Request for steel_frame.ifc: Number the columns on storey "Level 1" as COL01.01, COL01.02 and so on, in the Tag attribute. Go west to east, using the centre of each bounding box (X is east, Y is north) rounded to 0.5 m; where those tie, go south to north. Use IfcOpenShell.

First a look at what the model holds.

```python
import ifcopenshell
import ifcopenshell.util.element
import ifcopenshell.util.placement

model = ifcopenshell.open("steel_frame.ifc")
print(model.schema)
storey = next(s for s in model.by_type("IfcBuildingStorey") if s.Name == "Level 1")
columns = [e for e in ifcopenshell.util.element.get_decomposition(storey) if e.is_a("IfcColumn")]
for e in sorted(columns, key=lambda e: e.id()):
    origin = ifcopenshell.util.placement.get_local_placement(e.ObjectPlacement)[:3, 3]
    print(e.id(), e.Tag, e.Name, origin.round(2) + 0.0, sep=" | ")
```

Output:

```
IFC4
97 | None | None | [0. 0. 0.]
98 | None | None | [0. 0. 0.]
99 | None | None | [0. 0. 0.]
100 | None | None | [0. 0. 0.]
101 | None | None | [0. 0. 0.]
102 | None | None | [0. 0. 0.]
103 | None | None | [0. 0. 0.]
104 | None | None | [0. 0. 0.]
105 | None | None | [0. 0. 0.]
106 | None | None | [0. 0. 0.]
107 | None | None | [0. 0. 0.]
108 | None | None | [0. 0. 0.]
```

```python
import ifcopenshell
import ifcopenshell.geom
import ifcopenshell.util.element
import ifcopenshell.util.shape

model = ifcopenshell.open("steel_frame.ifc")
settings = ifcopenshell.geom.settings()
settings.set("use-world-coords", True)


def centre(element):
    shape = ifcopenshell.geom.create_shape(settings, element)
    return ifcopenshell.util.shape.get_bbox_centroid(shape.geometry)


storey = next(s for s in model.by_type("IfcBuildingStorey") if s.Name == "Level 1")
columns = [e for e in ifcopenshell.util.element.get_decomposition(storey) if e.is_a("IfcColumn")]

# Insertion points can sit at a corner or the storey origin, so sort by the geometry (in metres).
centres = {e: centre(e) for e in columns}
columns.sort(key=lambda e: (round(centres[e][0] / 0.5), centres[e][1]))

for i, e in enumerate(columns, start=1):
    number = f"COL01.{i:02d}"
    e.Tag = number
    print(e.id(), number)

model.write("steel_frame-out.ifc")
```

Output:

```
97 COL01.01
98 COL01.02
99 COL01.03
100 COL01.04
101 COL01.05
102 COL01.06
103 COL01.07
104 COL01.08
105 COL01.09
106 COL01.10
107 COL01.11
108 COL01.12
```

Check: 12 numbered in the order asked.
